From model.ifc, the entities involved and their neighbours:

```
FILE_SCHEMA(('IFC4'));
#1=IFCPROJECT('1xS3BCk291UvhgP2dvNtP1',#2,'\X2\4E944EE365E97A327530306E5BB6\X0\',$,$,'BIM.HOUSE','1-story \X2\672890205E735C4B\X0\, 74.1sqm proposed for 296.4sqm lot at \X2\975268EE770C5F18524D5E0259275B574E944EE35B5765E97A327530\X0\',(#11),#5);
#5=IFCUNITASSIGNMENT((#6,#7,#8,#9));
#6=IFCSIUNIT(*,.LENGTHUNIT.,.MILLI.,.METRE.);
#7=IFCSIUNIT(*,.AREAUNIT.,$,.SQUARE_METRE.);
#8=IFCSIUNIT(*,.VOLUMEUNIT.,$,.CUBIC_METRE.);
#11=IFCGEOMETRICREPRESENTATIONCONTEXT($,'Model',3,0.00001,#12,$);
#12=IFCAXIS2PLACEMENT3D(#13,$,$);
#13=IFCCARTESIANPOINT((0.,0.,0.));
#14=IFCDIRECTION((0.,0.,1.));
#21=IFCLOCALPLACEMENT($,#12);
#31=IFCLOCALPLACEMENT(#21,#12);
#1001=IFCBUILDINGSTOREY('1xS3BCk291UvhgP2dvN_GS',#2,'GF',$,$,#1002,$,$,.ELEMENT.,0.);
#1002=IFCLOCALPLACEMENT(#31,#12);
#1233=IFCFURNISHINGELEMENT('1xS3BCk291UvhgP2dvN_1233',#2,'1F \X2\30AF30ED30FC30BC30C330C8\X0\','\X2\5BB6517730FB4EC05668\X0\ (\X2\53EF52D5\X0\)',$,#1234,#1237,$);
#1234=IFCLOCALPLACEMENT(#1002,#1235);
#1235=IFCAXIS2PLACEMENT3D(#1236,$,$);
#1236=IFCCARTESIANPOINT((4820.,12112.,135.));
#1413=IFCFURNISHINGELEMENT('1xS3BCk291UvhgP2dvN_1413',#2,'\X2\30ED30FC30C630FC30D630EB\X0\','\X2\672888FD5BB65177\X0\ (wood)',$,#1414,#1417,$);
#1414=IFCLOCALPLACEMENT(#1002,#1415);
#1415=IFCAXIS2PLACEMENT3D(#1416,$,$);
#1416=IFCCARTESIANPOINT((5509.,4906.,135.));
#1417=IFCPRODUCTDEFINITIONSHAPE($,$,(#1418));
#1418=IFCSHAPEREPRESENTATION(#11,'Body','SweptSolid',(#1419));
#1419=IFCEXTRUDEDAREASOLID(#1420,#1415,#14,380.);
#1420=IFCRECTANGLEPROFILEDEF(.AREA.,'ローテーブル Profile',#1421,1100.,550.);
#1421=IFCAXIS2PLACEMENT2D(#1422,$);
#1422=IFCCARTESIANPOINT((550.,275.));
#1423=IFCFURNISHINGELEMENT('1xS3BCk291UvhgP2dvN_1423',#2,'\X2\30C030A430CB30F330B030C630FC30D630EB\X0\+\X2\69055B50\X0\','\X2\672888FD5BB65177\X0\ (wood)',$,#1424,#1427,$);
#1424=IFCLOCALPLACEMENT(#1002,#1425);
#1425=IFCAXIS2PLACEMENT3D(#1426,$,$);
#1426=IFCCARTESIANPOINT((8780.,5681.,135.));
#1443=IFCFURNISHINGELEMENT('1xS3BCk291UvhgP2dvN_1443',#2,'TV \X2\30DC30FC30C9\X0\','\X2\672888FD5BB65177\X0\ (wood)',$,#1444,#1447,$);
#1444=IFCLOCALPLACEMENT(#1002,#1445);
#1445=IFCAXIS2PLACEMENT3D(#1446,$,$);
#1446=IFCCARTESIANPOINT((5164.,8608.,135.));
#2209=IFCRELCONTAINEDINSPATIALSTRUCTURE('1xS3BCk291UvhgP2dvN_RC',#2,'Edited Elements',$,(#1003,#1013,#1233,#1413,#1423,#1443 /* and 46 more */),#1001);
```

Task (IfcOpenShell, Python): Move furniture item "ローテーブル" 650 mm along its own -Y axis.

```python
import ifcopenshell
import ifcopenshell.api.geometry
import ifcopenshell.util.placement
import ifcopenshell.util.unit

model = ifcopenshell.open("model.ifc")
unit_scale = ifcopenshell.util.unit.calculate_unit_scale(model)

item = model.by_guid("1xS3BCk291UvhgP2dvN_1413")
matrix = ifcopenshell.util.placement.get_local_placement(item.ObjectPlacement)
matrix[:3, 3] -= matrix[:3, 1] * 0.65 / unit_scale
ifcopenshell.api.geometry.edit_object_placement(model, product=item, matrix=matrix, is_si=False)

print(ifcopenshell.util.placement.get_local_placement(item.ObjectPlacement).round(3) + 0.0)

model.write("model-out.ifc")
```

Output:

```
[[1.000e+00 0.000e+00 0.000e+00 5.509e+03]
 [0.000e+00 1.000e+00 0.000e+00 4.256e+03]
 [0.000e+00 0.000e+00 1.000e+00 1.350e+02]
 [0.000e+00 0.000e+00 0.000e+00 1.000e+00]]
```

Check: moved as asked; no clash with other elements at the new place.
